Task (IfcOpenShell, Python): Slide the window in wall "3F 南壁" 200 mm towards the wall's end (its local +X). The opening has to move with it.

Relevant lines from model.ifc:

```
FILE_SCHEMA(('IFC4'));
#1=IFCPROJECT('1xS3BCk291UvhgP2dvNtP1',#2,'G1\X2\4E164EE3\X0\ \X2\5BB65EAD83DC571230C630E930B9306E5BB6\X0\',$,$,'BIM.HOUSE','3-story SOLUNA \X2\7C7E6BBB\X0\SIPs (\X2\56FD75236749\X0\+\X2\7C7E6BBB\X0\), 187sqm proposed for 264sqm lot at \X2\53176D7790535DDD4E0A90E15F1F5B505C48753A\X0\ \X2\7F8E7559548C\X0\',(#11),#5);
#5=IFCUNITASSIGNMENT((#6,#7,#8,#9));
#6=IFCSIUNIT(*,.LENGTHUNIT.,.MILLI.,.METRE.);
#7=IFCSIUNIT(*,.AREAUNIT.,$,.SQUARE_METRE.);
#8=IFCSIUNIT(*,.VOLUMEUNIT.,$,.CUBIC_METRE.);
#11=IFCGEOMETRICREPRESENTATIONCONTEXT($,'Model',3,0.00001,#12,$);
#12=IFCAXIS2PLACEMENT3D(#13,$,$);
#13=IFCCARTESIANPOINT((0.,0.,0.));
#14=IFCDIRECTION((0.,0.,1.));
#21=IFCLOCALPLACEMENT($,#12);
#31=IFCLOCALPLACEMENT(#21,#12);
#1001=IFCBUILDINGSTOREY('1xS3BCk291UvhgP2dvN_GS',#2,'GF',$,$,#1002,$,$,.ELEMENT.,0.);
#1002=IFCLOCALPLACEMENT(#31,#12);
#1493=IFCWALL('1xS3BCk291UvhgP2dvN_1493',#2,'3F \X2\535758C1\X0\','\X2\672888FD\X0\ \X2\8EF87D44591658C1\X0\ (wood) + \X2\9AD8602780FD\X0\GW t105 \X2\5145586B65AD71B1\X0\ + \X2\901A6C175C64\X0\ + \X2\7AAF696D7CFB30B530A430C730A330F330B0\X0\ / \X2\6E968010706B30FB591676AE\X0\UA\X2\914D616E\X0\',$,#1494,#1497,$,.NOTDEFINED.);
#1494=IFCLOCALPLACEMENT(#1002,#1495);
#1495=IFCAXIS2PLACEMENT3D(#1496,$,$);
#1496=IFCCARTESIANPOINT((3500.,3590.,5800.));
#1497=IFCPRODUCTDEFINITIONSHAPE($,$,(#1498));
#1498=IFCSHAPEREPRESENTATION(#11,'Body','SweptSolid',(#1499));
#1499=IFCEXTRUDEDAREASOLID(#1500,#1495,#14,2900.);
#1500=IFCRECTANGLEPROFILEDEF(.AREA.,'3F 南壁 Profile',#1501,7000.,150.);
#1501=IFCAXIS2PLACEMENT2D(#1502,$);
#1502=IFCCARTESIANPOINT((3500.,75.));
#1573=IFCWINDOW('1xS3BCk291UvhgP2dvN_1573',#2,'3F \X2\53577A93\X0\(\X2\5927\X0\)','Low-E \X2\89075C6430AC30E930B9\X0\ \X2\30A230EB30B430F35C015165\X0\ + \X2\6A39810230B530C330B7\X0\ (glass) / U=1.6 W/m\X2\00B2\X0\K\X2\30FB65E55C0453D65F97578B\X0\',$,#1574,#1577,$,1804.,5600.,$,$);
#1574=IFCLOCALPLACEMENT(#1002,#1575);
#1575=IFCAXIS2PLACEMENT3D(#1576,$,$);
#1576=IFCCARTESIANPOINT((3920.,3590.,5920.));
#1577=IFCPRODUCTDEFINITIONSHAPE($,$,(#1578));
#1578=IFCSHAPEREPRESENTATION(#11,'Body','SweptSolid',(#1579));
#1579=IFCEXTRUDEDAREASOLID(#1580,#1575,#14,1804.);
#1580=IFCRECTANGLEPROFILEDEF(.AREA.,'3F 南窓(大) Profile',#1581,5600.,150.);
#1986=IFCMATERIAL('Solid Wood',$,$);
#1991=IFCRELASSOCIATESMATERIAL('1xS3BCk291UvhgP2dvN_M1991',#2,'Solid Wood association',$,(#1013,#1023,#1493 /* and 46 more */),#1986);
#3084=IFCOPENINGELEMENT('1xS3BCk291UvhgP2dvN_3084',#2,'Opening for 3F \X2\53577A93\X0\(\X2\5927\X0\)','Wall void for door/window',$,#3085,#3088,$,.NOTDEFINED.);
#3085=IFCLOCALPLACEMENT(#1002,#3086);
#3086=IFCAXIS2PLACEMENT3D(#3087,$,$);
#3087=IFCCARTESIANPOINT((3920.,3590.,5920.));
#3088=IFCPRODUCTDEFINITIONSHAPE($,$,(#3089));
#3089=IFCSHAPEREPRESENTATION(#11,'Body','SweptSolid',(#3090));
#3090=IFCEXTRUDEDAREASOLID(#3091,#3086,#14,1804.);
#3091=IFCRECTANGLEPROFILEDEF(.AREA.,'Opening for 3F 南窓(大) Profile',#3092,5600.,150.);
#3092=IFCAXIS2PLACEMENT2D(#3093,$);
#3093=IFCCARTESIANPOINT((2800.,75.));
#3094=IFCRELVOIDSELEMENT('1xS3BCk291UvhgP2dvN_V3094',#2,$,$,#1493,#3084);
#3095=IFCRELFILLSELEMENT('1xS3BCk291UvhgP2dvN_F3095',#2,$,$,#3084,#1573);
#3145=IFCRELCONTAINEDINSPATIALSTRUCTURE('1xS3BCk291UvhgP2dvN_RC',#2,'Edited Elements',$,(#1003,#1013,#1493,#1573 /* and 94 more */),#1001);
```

```python
import ifcopenshell
import ifcopenshell.api.geometry
import ifcopenshell.util.placement
import ifcopenshell.util.unit

model = ifcopenshell.open("model.ifc")
unit_scale = ifcopenshell.util.unit.calculate_unit_scale(model)

window = model.by_guid("1xS3BCk291UvhgP2dvN_1573")
opening = window.FillsVoids[0].RelatingOpeningElement
wall = opening.VoidsElements[0].RelatingBuildingElement

wall_matrix = ifcopenshell.util.placement.get_local_placement(wall.ObjectPlacement)
shift = wall_matrix[:3, 0] * 0.2 / unit_scale
before = ifcopenshell.util.placement.get_local_placement(window.ObjectPlacement)[:3, 3].copy()

# The window is not placed relative to its opening, so move both.
for product in (opening, window):
    matrix = ifcopenshell.util.placement.get_local_placement(product.ObjectPlacement)
    matrix[:3, 3] += shift
    ifcopenshell.api.geometry.edit_object_placement(model, product=product, matrix=matrix, is_si=False)

after = ifcopenshell.util.placement.get_local_placement(window.ObjectPlacement)[:3, 3]
print("window moved by", (after - before).round(3) + 0.0)

model.write("model_edited.ifc")
```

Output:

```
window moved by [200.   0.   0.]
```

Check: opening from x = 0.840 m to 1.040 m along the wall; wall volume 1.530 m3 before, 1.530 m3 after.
